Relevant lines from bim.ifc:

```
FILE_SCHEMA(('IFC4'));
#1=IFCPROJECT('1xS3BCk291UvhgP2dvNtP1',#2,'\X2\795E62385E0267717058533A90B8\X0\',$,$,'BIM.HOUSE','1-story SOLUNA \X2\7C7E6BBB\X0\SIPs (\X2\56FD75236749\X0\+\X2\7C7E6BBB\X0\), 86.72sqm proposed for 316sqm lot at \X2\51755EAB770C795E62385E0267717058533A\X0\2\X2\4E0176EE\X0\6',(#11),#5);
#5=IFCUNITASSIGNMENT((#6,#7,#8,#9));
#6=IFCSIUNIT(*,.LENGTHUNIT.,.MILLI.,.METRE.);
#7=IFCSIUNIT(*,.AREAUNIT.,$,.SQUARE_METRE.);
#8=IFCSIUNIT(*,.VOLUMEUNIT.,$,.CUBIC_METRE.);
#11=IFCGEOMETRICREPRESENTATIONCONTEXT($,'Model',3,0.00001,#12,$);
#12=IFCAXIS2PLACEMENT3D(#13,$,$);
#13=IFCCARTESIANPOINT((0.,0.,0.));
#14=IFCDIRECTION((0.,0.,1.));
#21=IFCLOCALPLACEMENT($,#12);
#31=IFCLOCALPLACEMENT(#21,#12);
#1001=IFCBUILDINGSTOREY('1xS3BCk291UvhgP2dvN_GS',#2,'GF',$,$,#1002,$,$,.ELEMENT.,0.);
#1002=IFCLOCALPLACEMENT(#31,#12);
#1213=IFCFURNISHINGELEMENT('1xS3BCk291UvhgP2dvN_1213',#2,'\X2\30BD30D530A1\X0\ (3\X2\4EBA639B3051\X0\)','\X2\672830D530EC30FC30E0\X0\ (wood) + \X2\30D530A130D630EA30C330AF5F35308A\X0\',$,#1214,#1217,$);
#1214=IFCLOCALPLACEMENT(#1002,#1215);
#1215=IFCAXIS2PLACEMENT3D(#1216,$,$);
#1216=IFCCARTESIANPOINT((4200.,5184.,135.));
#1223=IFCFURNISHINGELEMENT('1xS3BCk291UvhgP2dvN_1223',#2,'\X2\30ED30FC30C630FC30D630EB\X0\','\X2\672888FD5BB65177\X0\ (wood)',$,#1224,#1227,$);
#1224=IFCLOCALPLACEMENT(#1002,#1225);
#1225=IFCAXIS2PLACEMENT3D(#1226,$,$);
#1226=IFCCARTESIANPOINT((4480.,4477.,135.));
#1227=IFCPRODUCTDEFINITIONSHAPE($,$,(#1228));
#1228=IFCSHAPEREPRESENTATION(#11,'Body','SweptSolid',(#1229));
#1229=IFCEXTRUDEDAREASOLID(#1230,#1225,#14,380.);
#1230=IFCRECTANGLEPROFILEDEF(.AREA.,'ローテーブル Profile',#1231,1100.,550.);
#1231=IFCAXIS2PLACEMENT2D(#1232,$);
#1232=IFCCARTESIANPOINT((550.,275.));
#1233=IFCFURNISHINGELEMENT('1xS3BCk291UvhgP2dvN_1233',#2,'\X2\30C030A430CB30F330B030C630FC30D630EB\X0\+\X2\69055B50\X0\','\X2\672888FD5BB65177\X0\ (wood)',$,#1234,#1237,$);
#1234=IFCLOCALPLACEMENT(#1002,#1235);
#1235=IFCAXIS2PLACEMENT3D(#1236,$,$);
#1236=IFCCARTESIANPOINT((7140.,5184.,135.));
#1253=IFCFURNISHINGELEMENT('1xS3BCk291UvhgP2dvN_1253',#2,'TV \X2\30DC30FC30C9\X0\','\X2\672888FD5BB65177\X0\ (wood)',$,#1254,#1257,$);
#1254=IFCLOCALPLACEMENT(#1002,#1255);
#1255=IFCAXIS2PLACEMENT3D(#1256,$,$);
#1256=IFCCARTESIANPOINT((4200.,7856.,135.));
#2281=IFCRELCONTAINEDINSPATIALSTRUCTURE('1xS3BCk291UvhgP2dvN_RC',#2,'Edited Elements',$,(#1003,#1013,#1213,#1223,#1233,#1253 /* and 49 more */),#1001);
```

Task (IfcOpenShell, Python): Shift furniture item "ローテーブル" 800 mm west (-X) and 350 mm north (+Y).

```python
import ifcopenshell
import ifcopenshell.api.geometry
import ifcopenshell.util.placement

model = ifcopenshell.open("bim.ifc")

item = model.by_guid("1xS3BCk291UvhgP2dvN_1223")
matrix = ifcopenshell.util.placement.get_local_placement(item.ObjectPlacement)
matrix[0, 3] -= 800.0
matrix[1, 3] += 350.0
ifcopenshell.api.geometry.edit_object_placement(model, product=item, matrix=matrix, is_si=False)

print(ifcopenshell.util.placement.get_local_placement(item.ObjectPlacement).round(3) + 0.0)

model.write("bim_edited.ifc")
```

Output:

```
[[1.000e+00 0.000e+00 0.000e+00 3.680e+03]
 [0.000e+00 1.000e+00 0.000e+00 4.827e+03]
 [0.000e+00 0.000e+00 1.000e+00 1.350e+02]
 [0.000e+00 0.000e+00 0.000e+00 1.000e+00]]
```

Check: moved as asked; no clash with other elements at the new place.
